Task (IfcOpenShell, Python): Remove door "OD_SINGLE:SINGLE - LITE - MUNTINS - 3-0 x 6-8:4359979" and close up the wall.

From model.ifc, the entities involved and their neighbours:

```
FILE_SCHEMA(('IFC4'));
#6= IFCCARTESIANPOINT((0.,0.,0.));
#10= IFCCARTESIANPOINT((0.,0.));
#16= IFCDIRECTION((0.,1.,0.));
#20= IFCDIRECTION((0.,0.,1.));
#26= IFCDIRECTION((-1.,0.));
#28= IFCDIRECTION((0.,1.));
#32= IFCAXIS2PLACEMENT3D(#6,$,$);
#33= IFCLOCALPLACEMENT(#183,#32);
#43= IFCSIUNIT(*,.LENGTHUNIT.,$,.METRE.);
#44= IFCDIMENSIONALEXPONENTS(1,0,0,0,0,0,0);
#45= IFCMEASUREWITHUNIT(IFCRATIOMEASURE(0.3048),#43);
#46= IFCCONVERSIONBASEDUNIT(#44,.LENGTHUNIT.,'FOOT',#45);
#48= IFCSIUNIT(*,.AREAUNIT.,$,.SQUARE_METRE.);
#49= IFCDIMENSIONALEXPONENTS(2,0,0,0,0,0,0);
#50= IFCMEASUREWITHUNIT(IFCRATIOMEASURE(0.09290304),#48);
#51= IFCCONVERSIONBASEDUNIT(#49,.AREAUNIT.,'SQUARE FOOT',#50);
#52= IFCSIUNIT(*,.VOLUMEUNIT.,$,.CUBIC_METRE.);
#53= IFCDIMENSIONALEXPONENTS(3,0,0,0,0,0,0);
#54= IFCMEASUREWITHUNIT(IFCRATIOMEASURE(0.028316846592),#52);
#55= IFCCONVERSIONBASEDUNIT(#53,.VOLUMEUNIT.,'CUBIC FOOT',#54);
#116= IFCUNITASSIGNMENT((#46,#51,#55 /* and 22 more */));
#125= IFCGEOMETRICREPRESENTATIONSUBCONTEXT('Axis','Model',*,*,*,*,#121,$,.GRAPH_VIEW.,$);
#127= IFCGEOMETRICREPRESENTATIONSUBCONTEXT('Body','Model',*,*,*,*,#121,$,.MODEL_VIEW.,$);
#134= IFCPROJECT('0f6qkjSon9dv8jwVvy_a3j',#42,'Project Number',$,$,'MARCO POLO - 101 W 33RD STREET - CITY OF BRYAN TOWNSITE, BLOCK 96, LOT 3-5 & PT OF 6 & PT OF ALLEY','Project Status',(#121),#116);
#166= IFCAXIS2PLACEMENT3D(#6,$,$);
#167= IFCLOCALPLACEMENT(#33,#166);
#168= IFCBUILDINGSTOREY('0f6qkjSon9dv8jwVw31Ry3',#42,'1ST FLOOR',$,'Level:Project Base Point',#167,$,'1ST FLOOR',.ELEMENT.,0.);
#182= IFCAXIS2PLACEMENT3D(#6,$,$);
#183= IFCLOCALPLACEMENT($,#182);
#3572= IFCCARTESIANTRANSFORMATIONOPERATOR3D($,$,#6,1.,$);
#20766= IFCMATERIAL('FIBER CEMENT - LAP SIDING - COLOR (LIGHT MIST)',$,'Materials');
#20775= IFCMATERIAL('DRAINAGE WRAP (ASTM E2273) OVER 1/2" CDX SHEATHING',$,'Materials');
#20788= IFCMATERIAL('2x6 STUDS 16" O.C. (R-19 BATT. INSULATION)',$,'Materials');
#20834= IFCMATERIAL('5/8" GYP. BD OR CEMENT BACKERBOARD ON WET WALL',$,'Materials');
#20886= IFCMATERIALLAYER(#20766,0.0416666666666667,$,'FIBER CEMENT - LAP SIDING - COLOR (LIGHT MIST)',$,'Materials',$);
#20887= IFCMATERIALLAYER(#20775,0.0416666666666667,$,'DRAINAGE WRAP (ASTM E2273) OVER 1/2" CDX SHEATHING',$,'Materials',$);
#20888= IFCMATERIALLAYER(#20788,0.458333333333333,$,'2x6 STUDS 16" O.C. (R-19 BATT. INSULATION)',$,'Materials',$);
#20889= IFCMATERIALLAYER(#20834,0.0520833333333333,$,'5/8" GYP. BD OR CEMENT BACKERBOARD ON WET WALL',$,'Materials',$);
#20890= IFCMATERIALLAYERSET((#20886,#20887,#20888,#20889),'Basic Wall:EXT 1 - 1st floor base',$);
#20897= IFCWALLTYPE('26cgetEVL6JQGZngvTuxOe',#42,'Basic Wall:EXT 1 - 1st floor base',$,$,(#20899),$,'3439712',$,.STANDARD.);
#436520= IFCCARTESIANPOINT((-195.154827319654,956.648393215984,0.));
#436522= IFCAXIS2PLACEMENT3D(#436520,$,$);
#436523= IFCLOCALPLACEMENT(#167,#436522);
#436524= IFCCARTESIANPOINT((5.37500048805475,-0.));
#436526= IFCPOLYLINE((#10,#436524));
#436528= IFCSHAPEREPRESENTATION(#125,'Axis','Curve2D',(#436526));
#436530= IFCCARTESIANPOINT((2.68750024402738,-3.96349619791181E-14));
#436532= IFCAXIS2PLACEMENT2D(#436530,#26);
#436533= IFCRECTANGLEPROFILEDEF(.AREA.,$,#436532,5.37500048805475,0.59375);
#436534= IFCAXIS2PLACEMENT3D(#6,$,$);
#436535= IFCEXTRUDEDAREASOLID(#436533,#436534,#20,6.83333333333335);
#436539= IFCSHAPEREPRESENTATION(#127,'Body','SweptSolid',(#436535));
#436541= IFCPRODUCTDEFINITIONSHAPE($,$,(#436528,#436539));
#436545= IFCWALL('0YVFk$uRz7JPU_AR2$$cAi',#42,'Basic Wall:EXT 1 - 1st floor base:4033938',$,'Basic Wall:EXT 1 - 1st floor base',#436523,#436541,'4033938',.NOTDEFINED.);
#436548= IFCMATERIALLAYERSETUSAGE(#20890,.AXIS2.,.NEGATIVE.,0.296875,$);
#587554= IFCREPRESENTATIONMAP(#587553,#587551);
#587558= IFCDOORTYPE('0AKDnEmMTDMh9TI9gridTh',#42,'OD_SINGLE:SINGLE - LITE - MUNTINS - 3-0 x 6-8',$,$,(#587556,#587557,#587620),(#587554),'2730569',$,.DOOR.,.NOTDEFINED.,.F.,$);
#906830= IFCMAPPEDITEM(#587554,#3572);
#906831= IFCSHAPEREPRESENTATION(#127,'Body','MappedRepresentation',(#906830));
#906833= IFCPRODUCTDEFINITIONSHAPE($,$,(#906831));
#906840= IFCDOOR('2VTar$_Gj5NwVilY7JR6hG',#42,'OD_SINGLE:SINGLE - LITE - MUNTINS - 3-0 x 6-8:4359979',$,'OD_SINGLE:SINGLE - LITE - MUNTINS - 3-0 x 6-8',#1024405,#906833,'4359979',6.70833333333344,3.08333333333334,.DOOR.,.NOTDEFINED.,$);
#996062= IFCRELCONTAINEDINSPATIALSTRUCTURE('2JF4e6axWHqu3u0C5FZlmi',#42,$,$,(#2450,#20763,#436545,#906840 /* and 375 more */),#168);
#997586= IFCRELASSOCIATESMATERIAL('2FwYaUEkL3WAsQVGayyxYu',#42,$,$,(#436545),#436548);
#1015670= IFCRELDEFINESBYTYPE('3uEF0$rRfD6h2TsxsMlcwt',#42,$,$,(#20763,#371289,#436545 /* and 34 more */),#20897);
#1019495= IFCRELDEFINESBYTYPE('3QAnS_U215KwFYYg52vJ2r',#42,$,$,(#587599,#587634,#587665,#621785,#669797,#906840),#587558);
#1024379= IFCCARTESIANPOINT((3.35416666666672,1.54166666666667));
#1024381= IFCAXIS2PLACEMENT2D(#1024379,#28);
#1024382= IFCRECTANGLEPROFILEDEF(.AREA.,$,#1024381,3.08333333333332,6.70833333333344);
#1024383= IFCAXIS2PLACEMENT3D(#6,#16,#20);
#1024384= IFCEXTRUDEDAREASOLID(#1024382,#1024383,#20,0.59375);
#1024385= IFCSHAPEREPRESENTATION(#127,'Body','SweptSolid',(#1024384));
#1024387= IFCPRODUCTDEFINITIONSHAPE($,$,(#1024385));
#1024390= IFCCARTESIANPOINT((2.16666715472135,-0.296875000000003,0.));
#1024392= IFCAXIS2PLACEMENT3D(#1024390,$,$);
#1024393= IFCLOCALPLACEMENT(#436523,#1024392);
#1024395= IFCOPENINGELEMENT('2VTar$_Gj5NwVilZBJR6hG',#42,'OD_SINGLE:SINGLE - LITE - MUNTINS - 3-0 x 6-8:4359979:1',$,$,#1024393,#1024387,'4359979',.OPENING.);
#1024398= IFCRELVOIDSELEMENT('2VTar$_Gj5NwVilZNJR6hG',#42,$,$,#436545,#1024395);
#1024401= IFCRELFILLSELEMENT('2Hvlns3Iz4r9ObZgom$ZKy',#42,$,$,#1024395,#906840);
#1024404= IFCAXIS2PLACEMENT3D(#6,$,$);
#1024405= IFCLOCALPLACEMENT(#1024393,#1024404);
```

```python
import ifcopenshell
import ifcopenshell.api.feature
import ifcopenshell.api.root
import ifcopenshell.geom
import ifcopenshell.util.shape

model = ifcopenshell.open("model.ifc")
settings = ifcopenshell.geom.settings()


def volume(element):
    """Net volume in cubic metres, openings subtracted."""
    shape = ifcopenshell.geom.create_shape(settings, element)
    return ifcopenshell.util.shape.get_volume(shape.geometry)


door = model.by_guid("2VTar$_Gj5NwVilY7JR6hG")
opening = door.FillsVoids[0].RelatingOpeningElement
wall = opening.VoidsElements[0].RelatingBuildingElement
before = volume(wall)

ifcopenshell.api.root.remove_product(model, product=door)
ifcopenshell.api.feature.remove_feature(model, feature=opening)

after = volume(wall)

print(f"wall volume {before:.3f} -> {after:.3f} m3")

model.write("model_edited.ifc")
```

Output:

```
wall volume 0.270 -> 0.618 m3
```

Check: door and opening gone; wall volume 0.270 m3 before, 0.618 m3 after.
